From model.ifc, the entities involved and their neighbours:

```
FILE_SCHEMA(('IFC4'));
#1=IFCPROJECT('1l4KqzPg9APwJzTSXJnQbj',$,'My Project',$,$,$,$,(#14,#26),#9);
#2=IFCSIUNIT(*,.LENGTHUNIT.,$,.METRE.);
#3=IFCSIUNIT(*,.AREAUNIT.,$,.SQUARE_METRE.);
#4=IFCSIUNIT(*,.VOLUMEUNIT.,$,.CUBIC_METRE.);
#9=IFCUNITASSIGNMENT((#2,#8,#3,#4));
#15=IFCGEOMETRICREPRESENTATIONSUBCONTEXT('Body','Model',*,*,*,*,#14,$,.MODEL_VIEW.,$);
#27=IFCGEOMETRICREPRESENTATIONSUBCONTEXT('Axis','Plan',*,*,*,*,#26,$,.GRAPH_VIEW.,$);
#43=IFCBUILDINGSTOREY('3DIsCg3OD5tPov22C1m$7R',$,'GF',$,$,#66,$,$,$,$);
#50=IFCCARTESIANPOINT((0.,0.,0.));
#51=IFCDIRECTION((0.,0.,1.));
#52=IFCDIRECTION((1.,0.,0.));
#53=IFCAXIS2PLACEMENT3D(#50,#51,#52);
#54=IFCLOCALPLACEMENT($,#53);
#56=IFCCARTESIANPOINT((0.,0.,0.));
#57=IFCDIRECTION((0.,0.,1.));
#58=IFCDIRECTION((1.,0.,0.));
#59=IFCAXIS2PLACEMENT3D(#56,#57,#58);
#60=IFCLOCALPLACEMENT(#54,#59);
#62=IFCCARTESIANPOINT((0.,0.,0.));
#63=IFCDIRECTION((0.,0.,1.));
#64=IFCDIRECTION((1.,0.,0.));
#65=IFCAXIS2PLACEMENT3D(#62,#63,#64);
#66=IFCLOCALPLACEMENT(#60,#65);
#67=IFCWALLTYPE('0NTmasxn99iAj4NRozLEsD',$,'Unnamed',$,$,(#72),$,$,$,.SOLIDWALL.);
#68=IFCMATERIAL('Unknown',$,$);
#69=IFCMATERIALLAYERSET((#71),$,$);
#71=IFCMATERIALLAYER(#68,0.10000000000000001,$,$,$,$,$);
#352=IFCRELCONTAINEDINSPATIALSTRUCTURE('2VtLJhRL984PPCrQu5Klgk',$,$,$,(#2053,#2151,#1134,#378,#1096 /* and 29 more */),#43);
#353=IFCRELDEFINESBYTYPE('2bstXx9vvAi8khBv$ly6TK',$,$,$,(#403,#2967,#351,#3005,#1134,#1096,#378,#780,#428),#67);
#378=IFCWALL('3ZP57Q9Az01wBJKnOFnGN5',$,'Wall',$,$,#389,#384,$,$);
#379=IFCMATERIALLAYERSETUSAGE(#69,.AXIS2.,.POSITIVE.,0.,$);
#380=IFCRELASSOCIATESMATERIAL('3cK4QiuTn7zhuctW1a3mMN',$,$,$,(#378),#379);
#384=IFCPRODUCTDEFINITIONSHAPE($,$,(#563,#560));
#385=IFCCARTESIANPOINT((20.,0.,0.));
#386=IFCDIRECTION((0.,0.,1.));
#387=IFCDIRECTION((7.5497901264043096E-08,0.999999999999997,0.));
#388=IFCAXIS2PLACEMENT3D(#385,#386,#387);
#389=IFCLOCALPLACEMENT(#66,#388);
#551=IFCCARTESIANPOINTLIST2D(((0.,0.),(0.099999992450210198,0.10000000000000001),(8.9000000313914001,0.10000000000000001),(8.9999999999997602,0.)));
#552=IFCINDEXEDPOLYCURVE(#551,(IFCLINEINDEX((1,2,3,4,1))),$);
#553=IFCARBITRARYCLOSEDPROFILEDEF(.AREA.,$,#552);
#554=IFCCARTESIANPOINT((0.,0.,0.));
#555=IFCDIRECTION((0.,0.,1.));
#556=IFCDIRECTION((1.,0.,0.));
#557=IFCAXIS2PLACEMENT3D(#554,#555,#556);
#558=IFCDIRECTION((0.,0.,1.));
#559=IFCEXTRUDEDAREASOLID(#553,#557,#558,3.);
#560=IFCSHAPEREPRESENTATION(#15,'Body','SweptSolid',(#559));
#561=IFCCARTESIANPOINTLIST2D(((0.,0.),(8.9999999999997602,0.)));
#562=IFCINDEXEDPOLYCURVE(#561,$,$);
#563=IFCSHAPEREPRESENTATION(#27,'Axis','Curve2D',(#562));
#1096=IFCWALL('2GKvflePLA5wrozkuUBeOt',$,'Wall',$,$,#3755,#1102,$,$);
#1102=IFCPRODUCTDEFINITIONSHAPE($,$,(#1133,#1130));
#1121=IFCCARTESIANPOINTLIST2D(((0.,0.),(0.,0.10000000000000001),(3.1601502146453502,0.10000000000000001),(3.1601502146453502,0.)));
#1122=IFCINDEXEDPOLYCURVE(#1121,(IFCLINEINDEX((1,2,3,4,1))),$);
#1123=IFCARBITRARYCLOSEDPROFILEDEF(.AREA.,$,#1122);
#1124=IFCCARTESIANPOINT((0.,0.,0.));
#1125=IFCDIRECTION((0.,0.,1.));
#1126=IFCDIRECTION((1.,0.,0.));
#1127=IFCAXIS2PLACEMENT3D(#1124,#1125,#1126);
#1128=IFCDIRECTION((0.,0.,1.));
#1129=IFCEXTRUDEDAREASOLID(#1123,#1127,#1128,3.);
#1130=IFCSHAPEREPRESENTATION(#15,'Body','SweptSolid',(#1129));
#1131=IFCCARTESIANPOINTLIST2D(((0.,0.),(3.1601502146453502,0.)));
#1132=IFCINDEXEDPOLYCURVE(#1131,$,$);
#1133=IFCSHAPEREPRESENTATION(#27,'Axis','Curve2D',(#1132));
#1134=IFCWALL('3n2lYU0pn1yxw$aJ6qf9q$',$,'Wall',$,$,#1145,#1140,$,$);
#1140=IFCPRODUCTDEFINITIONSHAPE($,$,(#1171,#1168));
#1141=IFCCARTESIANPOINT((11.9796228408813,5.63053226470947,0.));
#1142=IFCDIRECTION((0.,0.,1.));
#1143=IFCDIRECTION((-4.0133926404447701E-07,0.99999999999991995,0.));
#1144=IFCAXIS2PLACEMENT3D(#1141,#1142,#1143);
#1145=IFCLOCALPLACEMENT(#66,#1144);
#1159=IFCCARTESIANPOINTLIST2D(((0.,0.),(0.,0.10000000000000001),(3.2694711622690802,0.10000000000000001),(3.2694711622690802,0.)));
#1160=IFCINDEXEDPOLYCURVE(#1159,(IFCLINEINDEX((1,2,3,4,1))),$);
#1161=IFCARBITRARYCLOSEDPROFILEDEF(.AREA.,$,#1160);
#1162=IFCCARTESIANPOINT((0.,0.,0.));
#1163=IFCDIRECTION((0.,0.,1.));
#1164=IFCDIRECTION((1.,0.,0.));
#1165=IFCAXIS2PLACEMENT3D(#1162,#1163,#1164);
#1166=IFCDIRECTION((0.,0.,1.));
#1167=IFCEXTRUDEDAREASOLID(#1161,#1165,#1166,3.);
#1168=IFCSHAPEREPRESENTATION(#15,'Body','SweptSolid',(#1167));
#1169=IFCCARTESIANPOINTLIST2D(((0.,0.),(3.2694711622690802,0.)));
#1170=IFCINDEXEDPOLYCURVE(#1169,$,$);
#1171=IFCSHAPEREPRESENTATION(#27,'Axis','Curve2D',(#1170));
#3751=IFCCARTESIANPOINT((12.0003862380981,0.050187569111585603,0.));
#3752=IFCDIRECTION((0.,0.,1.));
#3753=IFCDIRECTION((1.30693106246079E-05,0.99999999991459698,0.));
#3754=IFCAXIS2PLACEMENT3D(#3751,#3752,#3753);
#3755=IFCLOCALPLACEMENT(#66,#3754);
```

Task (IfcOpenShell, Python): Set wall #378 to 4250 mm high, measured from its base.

```python
import ifcopenshell
import ifcopenshell.geom
import ifcopenshell.util.representation
import ifcopenshell.util.shape
import ifcopenshell.util.unit

model = ifcopenshell.open("model.ifc")
unit_scale = ifcopenshell.util.unit.calculate_unit_scale(model)
settings = ifcopenshell.geom.settings()


def volume(element):
    """Net volume in cubic metres, openings subtracted."""
    shape = ifcopenshell.geom.create_shape(settings, element)
    return ifcopenshell.util.shape.get_volume(shape.geometry)


wall = model.by_guid("3ZP57Q9Az01wBJKnOFnGN5")
before = volume(wall)

body = ifcopenshell.util.representation.get_representation(wall, "Model", "Body")
solid = body.Items[0]
old_height = solid.Depth
solid.Depth = 4.25 / unit_scale
after = volume(wall)

print(f"height {old_height:g} -> {solid.Depth:g}, volume {before:.3f} -> {after:.3f} m3")

model.write("model_edited.ifc")
```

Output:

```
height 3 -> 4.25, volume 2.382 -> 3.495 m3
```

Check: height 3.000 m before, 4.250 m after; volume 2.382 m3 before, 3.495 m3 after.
